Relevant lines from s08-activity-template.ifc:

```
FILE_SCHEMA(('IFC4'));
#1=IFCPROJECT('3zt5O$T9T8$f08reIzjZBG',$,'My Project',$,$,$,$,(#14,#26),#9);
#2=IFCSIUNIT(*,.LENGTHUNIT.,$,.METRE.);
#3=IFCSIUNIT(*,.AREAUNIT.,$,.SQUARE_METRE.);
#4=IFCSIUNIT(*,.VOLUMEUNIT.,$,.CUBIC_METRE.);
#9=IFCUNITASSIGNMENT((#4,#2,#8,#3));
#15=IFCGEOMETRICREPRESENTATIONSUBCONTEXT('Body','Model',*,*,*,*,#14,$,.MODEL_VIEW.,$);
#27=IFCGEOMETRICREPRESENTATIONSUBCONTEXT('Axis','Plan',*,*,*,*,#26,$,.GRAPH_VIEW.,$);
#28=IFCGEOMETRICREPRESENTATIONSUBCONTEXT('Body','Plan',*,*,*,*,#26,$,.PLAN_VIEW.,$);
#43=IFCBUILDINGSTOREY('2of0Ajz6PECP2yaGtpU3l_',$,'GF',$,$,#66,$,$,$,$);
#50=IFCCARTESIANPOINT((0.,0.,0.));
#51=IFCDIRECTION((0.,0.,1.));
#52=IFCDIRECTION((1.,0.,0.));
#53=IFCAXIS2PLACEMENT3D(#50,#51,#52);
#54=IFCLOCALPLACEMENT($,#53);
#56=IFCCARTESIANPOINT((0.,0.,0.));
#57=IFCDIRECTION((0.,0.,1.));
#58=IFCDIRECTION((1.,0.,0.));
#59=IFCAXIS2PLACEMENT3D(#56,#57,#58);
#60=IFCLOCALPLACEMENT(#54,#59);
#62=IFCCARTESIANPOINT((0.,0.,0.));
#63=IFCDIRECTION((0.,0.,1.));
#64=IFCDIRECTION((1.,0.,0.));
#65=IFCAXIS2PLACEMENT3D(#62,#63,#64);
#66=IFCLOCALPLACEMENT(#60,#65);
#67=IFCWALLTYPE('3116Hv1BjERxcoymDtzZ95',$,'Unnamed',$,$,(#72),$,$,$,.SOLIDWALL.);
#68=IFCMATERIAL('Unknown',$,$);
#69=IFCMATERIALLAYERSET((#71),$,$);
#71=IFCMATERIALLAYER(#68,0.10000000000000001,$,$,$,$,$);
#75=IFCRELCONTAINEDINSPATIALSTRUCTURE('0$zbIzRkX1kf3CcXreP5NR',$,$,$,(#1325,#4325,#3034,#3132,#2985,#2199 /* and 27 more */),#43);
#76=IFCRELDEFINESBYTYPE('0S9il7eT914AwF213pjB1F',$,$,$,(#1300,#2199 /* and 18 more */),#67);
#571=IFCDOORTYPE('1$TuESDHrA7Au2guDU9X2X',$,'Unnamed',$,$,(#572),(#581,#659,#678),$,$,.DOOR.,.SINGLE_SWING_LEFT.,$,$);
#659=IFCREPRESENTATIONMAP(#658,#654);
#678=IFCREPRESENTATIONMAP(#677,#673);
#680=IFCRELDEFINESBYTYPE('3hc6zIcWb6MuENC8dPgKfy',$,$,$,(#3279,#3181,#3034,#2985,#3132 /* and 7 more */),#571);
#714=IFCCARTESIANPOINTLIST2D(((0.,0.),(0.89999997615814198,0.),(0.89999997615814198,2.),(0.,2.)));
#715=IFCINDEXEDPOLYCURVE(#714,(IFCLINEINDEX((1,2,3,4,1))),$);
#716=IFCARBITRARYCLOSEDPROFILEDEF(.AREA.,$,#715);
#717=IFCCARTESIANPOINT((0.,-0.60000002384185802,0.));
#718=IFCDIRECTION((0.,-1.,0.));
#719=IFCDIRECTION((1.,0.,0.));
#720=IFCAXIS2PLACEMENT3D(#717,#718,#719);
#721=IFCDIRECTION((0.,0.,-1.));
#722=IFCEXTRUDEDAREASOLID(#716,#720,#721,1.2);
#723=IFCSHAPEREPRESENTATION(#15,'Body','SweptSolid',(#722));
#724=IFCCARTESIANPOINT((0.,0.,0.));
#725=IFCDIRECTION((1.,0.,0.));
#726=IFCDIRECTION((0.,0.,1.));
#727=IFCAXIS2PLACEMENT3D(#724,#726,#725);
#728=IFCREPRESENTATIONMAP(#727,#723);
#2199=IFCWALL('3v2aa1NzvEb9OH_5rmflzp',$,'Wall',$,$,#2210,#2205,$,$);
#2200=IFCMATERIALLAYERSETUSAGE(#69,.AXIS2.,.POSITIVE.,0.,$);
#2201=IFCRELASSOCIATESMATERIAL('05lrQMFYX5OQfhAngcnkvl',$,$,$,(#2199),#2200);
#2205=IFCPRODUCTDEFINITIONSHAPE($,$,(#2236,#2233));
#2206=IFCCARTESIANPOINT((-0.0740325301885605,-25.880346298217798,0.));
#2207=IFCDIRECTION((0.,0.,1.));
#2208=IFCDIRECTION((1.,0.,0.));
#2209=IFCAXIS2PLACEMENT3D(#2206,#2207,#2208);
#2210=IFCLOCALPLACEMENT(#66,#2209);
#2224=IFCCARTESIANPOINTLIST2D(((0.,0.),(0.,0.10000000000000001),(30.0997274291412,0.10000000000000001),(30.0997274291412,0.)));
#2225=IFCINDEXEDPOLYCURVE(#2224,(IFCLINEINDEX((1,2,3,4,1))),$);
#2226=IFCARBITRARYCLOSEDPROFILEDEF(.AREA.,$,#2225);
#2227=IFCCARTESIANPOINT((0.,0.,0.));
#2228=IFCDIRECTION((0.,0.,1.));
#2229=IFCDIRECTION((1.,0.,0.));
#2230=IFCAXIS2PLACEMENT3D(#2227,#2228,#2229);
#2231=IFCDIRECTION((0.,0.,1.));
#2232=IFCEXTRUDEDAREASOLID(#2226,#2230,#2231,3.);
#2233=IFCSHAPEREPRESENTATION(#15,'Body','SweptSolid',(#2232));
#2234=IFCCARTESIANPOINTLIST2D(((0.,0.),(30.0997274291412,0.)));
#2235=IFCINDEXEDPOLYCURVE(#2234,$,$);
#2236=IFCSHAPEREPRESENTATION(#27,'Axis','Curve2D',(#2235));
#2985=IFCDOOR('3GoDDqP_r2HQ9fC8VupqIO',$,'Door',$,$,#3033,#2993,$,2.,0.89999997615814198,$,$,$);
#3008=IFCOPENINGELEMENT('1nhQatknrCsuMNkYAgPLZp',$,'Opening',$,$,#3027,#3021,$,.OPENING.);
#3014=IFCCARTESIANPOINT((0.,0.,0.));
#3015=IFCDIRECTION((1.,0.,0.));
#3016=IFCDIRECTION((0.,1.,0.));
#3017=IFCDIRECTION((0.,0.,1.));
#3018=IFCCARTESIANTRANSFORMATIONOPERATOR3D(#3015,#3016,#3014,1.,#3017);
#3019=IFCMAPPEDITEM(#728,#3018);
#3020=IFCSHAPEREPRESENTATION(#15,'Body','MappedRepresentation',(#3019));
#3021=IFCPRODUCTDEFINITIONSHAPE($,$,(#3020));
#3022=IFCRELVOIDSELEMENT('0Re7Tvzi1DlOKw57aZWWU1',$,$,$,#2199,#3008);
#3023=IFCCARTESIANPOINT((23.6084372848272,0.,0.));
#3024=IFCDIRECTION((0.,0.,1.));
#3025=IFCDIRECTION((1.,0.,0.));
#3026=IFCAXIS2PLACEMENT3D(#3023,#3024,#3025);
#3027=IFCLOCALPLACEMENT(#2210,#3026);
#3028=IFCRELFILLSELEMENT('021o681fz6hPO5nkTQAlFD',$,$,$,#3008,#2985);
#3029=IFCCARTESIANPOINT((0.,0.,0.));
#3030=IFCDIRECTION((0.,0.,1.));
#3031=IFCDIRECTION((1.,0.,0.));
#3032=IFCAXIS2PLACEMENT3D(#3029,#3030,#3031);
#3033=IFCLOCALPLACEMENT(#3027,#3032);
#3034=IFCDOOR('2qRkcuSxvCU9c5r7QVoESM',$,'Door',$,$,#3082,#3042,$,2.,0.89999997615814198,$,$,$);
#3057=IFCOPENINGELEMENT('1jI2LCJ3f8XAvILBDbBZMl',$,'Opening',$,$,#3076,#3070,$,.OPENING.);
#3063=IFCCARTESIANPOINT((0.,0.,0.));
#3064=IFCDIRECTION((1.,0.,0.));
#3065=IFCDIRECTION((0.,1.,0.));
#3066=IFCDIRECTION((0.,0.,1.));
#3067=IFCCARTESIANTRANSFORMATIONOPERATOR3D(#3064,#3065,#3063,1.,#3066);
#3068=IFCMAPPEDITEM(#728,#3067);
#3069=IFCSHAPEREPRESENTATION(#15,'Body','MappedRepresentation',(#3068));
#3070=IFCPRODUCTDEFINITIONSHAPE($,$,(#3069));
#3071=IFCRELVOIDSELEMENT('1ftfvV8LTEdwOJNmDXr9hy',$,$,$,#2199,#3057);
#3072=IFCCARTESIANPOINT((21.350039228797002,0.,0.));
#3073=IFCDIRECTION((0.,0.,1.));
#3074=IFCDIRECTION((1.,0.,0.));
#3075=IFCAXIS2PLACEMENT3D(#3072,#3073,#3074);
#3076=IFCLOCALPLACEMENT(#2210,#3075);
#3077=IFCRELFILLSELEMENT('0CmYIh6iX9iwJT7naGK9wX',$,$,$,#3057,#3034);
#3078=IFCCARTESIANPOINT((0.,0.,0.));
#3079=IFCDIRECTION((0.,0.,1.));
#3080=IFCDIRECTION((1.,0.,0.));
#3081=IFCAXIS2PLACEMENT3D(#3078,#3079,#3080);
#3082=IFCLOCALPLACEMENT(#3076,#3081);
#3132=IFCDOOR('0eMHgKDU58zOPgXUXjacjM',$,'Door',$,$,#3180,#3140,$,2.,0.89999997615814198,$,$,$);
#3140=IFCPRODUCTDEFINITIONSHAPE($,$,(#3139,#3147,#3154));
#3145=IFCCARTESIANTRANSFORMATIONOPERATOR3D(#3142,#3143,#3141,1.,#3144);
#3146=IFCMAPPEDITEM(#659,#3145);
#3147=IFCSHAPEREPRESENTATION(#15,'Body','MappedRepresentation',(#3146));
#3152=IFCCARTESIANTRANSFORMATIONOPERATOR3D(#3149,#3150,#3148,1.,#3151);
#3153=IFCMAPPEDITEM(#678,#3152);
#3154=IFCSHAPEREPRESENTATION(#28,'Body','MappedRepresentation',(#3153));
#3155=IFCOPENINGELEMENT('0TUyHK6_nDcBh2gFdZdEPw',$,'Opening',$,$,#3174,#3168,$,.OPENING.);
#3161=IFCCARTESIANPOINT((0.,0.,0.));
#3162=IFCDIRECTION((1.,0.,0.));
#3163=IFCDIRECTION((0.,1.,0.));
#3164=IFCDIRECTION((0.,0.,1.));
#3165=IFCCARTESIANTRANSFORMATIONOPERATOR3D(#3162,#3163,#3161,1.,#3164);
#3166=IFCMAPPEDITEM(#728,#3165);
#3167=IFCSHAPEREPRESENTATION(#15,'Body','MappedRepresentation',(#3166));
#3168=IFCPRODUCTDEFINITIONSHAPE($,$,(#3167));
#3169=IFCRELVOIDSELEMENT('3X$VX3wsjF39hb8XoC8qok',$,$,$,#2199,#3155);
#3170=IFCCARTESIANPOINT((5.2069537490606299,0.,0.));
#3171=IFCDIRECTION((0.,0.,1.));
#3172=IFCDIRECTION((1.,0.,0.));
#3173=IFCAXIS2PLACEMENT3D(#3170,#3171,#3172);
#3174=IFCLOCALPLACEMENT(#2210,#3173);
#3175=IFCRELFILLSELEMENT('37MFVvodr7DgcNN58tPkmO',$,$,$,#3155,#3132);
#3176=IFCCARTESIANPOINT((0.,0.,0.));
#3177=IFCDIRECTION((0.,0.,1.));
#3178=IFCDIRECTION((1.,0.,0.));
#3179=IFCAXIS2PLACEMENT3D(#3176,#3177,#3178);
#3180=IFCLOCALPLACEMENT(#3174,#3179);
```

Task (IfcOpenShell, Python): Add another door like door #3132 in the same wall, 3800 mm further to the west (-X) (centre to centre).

```python
import ifcopenshell
import ifcopenshell.api.feature
import ifcopenshell.api.geometry
import ifcopenshell.api.root
import ifcopenshell.geom
import ifcopenshell.util.element
import ifcopenshell.util.placement
import ifcopenshell.util.shape

model = ifcopenshell.open("s08-activity-template.ifc")
settings = ifcopenshell.geom.settings()


def volume(element):
    """Net volume in cubic metres, openings subtracted."""
    shape = ifcopenshell.geom.create_shape(settings, element)
    return ifcopenshell.util.shape.get_volume(shape.geometry)


door = model.by_id(3132)
opening = door.FillsVoids[0].RelatingOpeningElement
wall = opening.VoidsElements[0].RelatingBuildingElement
before = volume(wall)
shift = ifcopenshell.util.placement.get_local_placement(wall.ObjectPlacement)[:3, 0] * -3.8

# copy_class copies the void relationship, type, container and properties, but no geometry.
new_opening = ifcopenshell.api.root.copy_class(model, product=opening)
new_opening.Representation = ifcopenshell.util.element.copy_deep(
    model, opening.Representation, exclude=["IfcGeometricRepresentationContext", "IfcRepresentationMap"]
)
new_door = ifcopenshell.api.root.copy_class(model, product=door)
new_door.Representation = ifcopenshell.util.element.copy_deep(
    model, door.Representation, exclude=["IfcGeometricRepresentationContext", "IfcRepresentationMap"]
)
ifcopenshell.api.feature.add_filling(model, opening=new_opening, element=new_door)

for old, new in ((opening, new_opening), (door, new_door)):
    matrix = ifcopenshell.util.placement.get_local_placement(old.ObjectPlacement)
    matrix[:3, 3] += shift
    ifcopenshell.api.geometry.edit_object_placement(model, product=new, matrix=matrix, is_si=False)

after = volume(wall)

print(f"wall volume {before:.3f} -> {after:.3f} m3")

model.write("s08-activity-template-out.ifc")
```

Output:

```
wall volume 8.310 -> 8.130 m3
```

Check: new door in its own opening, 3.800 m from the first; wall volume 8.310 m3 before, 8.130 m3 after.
